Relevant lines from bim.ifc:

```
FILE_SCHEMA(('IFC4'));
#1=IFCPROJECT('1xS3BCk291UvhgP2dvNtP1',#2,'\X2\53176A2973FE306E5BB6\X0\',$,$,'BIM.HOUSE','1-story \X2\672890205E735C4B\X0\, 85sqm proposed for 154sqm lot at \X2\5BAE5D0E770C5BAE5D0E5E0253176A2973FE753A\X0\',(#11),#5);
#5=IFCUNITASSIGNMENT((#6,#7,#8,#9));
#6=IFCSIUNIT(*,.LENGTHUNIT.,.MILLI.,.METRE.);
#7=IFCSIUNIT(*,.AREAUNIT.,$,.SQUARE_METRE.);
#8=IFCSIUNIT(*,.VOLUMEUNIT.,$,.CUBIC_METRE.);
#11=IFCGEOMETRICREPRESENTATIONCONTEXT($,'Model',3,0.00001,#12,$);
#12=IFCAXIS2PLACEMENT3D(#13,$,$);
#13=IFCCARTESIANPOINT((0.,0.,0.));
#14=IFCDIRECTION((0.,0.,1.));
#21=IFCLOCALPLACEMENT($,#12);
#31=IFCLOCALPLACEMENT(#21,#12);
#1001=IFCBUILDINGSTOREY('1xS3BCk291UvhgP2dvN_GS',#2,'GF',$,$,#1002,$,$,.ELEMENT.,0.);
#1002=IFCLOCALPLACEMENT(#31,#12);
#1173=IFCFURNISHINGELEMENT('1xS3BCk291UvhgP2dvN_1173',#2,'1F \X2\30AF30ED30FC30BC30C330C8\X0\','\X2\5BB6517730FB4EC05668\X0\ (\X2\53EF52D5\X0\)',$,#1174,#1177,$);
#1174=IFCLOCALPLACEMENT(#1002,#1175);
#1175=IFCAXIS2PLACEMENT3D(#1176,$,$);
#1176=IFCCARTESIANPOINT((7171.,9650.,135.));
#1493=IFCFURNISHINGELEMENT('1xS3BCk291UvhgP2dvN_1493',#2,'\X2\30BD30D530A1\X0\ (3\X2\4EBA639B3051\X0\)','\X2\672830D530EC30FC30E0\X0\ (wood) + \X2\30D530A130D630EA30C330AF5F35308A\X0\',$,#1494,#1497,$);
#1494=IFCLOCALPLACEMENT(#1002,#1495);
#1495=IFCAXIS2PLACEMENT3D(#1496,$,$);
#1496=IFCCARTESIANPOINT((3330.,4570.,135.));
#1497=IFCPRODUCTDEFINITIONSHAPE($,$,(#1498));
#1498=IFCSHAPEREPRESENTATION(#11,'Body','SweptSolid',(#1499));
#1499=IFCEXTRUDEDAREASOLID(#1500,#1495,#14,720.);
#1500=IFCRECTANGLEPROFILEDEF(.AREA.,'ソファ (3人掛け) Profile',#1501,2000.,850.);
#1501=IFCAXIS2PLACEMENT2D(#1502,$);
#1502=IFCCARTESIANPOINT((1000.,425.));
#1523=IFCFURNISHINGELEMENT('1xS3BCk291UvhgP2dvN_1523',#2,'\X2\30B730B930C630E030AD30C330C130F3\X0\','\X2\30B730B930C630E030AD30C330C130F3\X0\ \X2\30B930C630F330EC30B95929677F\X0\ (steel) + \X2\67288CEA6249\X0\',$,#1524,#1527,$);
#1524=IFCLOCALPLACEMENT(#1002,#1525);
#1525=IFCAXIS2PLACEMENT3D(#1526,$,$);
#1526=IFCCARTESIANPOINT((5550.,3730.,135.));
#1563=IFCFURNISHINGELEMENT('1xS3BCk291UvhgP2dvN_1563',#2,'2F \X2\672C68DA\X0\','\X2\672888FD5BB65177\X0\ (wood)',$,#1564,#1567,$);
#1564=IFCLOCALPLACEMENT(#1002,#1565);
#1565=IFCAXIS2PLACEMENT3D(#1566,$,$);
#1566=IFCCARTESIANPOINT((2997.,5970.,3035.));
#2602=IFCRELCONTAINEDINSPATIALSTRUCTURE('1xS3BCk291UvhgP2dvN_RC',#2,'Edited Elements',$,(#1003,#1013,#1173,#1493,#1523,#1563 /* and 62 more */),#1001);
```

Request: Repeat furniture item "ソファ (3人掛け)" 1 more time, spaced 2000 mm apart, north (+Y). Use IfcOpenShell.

```python
import numpy as np
import ifcopenshell
import ifcopenshell.api.geometry
import ifcopenshell.api.root
import ifcopenshell.util.element
import ifcopenshell.util.placement

model = ifcopenshell.open("bim.ifc")


def reuse_history(source, copy):
    """copy_class also copies each property set's owner history, people and application; keep the originals."""
    for rel in copy.IsDefinedBy:
        if rel.is_a("IfcRelDefinesByProperties") and (history := rel.RelatingPropertyDefinition.OwnerHistory):
            rel.RelatingPropertyDefinition.OwnerHistory = source.OwnerHistory
            ifcopenshell.util.element.remove_deep2(model, history)


source = model.by_guid("1xS3BCk291UvhgP2dvN_1493")
base = ifcopenshell.util.placement.get_local_placement(source.ObjectPlacement)
step = np.array([0.0, 1.0, 0.0]) * 2000.0

for i in range(1, 2):
    copy = ifcopenshell.api.root.copy_class(model, product=source)
    copy.Representation = ifcopenshell.util.element.copy_deep(
        model, source.Representation, exclude=["IfcGeometricRepresentationContext", "IfcRepresentationMap"]
    )
    reuse_history(source, copy)
    matrix = base.copy()
    matrix[:3, 3] += i * step
    print("added at", matrix[:3, 3].round(3) + 0.0)
    ifcopenshell.api.geometry.edit_object_placement(model, product=copy, matrix=matrix, is_si=False)

model.write("bim_v2.ifc")
```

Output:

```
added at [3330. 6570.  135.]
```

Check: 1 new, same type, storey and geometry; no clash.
